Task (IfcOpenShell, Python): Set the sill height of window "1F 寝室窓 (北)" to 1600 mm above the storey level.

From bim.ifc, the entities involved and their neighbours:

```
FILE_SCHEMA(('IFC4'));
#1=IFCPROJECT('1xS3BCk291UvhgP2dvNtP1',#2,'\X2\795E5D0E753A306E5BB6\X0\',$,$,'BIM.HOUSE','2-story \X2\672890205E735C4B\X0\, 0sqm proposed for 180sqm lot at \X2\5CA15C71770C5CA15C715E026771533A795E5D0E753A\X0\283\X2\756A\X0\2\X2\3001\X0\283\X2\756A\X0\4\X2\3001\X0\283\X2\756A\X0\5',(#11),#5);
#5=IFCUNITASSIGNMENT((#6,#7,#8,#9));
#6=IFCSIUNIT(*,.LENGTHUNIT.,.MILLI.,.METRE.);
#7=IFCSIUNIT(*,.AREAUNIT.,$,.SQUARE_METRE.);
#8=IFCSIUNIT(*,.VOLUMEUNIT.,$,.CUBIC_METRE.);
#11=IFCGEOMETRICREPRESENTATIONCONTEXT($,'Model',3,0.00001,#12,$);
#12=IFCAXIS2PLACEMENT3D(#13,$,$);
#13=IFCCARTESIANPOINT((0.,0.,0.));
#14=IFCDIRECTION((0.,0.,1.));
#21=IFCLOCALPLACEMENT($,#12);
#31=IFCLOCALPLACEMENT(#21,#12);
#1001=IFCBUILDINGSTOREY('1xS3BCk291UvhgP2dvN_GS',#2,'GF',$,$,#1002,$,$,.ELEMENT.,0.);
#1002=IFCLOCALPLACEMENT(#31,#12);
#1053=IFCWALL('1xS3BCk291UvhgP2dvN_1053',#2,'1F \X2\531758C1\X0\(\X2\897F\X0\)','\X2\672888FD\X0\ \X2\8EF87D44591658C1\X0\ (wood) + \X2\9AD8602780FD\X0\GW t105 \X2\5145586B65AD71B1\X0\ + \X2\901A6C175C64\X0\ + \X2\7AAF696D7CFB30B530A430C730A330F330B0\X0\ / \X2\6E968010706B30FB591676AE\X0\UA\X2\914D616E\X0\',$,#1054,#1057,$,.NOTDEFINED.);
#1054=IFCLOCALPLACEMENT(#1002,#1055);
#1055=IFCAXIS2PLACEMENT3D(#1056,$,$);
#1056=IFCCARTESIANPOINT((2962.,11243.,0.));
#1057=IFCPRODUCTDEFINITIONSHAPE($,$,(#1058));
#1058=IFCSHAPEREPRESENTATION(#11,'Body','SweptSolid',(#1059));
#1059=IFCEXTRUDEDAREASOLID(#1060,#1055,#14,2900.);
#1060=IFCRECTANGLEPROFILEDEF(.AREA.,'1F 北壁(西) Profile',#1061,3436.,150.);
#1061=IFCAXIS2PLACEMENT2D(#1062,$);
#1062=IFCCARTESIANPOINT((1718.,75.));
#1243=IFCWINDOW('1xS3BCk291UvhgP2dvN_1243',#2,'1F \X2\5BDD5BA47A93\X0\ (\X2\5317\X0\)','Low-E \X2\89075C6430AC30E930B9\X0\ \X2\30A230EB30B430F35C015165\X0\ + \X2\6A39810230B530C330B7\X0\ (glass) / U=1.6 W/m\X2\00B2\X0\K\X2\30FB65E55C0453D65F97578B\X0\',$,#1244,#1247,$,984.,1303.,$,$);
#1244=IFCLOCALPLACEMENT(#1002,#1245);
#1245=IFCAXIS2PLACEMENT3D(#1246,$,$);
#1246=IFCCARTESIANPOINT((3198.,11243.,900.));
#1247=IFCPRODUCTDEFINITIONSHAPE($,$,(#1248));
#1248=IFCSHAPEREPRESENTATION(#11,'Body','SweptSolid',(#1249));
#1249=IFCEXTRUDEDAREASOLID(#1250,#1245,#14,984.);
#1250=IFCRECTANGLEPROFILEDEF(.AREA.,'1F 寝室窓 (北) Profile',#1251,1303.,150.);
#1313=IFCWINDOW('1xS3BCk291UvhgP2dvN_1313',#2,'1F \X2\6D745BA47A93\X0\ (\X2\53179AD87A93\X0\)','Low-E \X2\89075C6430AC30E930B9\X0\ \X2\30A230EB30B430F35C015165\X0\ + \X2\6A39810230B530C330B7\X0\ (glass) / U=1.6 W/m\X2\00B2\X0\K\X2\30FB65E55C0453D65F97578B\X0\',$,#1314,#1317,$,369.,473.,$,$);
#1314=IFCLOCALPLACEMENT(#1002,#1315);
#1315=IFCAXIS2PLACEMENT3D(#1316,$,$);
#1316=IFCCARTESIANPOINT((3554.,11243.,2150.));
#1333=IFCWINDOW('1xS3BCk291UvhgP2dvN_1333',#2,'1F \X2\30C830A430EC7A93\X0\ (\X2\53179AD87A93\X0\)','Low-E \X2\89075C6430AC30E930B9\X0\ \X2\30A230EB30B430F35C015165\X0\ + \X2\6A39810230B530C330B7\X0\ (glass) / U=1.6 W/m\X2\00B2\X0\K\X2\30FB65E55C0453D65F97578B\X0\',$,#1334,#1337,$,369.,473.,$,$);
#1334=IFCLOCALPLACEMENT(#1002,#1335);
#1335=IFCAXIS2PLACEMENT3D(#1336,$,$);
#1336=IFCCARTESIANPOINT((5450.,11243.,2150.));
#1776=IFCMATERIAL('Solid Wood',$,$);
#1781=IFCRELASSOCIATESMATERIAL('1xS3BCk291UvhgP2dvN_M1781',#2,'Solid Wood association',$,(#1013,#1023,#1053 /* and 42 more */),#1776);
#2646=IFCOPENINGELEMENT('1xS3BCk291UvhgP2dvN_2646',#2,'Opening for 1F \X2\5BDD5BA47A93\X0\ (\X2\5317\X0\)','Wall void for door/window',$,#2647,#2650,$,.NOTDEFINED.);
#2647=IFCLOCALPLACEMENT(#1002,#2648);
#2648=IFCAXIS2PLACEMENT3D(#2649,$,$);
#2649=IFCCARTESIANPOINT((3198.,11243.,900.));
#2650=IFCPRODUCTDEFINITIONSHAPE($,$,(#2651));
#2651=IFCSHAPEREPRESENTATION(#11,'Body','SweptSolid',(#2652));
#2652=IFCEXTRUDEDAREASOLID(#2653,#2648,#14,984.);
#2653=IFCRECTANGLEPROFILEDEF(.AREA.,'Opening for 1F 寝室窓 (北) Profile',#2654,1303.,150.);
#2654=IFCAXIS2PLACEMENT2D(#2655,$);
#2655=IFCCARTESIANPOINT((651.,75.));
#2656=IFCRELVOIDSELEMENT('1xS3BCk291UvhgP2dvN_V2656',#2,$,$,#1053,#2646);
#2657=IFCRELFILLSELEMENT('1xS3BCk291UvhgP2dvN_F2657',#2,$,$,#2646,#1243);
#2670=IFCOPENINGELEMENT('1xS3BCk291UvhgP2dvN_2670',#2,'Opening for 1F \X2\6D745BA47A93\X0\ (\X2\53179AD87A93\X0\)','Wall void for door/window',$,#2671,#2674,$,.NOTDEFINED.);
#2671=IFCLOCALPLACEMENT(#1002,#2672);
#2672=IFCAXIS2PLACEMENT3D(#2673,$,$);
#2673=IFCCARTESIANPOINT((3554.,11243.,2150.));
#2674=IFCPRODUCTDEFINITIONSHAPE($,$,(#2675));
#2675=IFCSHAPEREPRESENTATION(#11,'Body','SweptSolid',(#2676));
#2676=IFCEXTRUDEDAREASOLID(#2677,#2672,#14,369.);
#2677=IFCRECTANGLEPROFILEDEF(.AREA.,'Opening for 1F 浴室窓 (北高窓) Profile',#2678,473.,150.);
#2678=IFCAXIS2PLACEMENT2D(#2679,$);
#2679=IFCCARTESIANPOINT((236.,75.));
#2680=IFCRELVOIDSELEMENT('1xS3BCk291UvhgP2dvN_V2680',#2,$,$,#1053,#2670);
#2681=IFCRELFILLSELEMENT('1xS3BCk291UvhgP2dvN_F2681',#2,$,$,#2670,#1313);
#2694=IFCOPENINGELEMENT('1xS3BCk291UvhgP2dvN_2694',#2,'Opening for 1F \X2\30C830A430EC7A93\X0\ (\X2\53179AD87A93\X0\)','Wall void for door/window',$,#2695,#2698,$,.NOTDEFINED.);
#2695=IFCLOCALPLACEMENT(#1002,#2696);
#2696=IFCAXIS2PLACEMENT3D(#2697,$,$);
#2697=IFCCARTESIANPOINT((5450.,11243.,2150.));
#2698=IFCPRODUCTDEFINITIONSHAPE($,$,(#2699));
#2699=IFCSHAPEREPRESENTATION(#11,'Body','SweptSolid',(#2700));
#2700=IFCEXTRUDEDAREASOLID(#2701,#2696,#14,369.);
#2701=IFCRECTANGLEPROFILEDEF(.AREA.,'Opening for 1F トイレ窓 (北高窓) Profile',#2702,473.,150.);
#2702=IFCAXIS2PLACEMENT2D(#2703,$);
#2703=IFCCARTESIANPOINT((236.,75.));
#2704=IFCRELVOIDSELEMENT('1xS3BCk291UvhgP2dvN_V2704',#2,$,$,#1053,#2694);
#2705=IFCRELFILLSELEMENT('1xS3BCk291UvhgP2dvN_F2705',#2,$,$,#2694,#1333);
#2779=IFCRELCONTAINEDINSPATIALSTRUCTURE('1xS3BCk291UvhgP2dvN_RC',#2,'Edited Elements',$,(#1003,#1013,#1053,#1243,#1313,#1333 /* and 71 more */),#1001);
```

```python
import numpy as np
import ifcopenshell
import ifcopenshell.api.geometry
import ifcopenshell.geom
import ifcopenshell.util.element
import ifcopenshell.util.placement
import ifcopenshell.util.shape
import ifcopenshell.util.unit

model = ifcopenshell.open("bim.ifc")
unit_scale = ifcopenshell.util.unit.calculate_unit_scale(model)

window = model.by_guid("1xS3BCk291UvhgP2dvN_1243")
opening = window.FillsVoids[0].RelatingOpeningElement
storey = ifcopenshell.util.element.get_container(window, ifc_class="IfcBuildingStorey")
level = ifcopenshell.util.placement.get_local_placement(storey.ObjectPlacement)[2, 3]

# The opening's origin need not be at the sill, so measure its lowest point.
shape = ifcopenshell.geom.create_shape(ifcopenshell.geom.settings(), opening)
bottom = ifcopenshell.util.shape.get_shape_bottom_elevation(shape, shape.geometry) / unit_scale
dz = level + 1.6 / unit_scale - bottom

shift = np.array([0.0, 0.0, dz])
# The window is not placed relative to its opening, so move both.
for product in (opening, window):
    matrix = ifcopenshell.util.placement.get_local_placement(product.ObjectPlacement)
    matrix[:3, 3] += shift
    ifcopenshell.api.geometry.edit_object_placement(model, product=product, matrix=matrix, is_si=False)

print(f"moved by {dz * unit_scale:+.3f} m")

model.write("bim_updated.ifc")
```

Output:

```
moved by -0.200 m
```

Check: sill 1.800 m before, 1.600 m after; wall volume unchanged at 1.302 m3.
